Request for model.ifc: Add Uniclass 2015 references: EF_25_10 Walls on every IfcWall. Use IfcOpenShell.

First a look at what the model holds.

```python
import ifcopenshell

model = ifcopenshell.open("model.ifc")
print(model.schema)
print("classifications:", [c.Name for c in model.by_type("IfcClassification")])
for ifc_class in ("IfcDoor", "IfcRoof", "IfcStair", "IfcWall", "IfcWindow"):
    print(ifc_class, len(model.by_type(ifc_class)))
```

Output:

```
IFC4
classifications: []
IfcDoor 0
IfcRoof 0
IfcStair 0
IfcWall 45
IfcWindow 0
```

```python
import ifcopenshell
import ifcopenshell.api.classification

model = ifcopenshell.open("model.ifc")

system = ifcopenshell.api.classification.add_classification(model, classification="Uniclass 2015")

codes = {
    "IfcWall": ("EF_25_10", "Walls"),
}
for ifc_class, (code, name) in codes.items():
    products = model.by_type(ifc_class)
    ifcopenshell.api.classification.add_reference(
        model, products=products, classification=system, identification=code, name=name
    )
    print(code, len(products))

model.write("model_edited.ifc")
```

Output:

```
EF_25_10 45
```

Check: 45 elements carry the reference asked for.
